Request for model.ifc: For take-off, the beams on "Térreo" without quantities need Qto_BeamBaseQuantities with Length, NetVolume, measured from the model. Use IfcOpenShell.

First a look at what the model holds.

```python
import ifcopenshell
import ifcopenshell.util.element
import ifcopenshell.util.unit

model = ifcopenshell.open("model.ifc")
print(model.schema)
for unit_type in ("LENGTHUNIT", "AREAUNIT", "VOLUMEUNIT"):
    print(unit_type, ifcopenshell.util.unit.calculate_unit_scale(model, unit_type))
storey = next(s for s in model.by_type("IfcBuildingStorey") if s.Name == "Térreo")
beams = [e for e in ifcopenshell.util.element.get_decomposition(storey) if e.is_a("IfcBeam")]
for e in sorted(beams, key=lambda e: e.id()):
    print(e.id(), e.is_a(), e.Name, list(ifcopenshell.util.element.get_psets(e, qtos_only=True)), sep=" | ")
```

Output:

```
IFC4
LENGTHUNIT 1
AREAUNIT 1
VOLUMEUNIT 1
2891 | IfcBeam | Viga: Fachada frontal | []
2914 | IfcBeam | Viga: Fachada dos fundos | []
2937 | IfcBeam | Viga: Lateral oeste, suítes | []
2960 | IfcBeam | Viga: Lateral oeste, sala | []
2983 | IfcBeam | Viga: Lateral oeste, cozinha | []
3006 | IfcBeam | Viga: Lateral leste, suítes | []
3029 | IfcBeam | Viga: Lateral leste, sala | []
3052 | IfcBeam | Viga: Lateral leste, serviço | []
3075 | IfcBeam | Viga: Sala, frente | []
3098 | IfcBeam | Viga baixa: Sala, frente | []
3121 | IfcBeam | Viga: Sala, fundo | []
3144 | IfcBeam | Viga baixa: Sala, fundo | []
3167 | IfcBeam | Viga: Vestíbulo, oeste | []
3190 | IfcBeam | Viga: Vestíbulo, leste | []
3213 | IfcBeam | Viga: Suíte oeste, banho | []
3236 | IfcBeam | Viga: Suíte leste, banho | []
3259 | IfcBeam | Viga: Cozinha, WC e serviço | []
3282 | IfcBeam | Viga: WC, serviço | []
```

```python
import ifcopenshell
import ifcopenshell.api.pset
import ifcopenshell.geom
import ifcopenshell.util.element
import ifcopenshell.util.shape
import ifcopenshell.util.unit

model = ifcopenshell.open("model.ifc")
unit_scale = ifcopenshell.util.unit.calculate_unit_scale(model)
volume_scale = ifcopenshell.util.unit.calculate_unit_scale(model, "VOLUMEUNIT")
settings = ifcopenshell.geom.settings()

storey = next(s for s in model.by_type("IfcBuildingStorey") if s.Name == "Térreo")
beams = [e for e in ifcopenshell.util.element.get_decomposition(storey) if e.is_a("IfcBeam")]

for e in sorted(beams, key=lambda e: e.id()):
    if ifcopenshell.util.element.get_psets(e, qtos_only=True, should_inherit=False):
        continue
    # Geometry comes back in metres, in the element's own axes.
    shape = ifcopenshell.geom.create_shape(settings, e)
    values = {
        "Length": ifcopenshell.util.shape.get_max_xyz(shape.geometry) / unit_scale,
        "NetVolume": ifcopenshell.util.shape.get_volume(shape.geometry) / volume_scale,
    }
    qto = ifcopenshell.api.pset.add_qto(model, product=e, name="Qto_BeamBaseQuantities")
    ifcopenshell.api.pset.edit_qto(model, qto=qto, properties=values)
    print(e.id(), {k: round(v, 3) for k, v in values.items()})

model.write("model_updated.ifc")
```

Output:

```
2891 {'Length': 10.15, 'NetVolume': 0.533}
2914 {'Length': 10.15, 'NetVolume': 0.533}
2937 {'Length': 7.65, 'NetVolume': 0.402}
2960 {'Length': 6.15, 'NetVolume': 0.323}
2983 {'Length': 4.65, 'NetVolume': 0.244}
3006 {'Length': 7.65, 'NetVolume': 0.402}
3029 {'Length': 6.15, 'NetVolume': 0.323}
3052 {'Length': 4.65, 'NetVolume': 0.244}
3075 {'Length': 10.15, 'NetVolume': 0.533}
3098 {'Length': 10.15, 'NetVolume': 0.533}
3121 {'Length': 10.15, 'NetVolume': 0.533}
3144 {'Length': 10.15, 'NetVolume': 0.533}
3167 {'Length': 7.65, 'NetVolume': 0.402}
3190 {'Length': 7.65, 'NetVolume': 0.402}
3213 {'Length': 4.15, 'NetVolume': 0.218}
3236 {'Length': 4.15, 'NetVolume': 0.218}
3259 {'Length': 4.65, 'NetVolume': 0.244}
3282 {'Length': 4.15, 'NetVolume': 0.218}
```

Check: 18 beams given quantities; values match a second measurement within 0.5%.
